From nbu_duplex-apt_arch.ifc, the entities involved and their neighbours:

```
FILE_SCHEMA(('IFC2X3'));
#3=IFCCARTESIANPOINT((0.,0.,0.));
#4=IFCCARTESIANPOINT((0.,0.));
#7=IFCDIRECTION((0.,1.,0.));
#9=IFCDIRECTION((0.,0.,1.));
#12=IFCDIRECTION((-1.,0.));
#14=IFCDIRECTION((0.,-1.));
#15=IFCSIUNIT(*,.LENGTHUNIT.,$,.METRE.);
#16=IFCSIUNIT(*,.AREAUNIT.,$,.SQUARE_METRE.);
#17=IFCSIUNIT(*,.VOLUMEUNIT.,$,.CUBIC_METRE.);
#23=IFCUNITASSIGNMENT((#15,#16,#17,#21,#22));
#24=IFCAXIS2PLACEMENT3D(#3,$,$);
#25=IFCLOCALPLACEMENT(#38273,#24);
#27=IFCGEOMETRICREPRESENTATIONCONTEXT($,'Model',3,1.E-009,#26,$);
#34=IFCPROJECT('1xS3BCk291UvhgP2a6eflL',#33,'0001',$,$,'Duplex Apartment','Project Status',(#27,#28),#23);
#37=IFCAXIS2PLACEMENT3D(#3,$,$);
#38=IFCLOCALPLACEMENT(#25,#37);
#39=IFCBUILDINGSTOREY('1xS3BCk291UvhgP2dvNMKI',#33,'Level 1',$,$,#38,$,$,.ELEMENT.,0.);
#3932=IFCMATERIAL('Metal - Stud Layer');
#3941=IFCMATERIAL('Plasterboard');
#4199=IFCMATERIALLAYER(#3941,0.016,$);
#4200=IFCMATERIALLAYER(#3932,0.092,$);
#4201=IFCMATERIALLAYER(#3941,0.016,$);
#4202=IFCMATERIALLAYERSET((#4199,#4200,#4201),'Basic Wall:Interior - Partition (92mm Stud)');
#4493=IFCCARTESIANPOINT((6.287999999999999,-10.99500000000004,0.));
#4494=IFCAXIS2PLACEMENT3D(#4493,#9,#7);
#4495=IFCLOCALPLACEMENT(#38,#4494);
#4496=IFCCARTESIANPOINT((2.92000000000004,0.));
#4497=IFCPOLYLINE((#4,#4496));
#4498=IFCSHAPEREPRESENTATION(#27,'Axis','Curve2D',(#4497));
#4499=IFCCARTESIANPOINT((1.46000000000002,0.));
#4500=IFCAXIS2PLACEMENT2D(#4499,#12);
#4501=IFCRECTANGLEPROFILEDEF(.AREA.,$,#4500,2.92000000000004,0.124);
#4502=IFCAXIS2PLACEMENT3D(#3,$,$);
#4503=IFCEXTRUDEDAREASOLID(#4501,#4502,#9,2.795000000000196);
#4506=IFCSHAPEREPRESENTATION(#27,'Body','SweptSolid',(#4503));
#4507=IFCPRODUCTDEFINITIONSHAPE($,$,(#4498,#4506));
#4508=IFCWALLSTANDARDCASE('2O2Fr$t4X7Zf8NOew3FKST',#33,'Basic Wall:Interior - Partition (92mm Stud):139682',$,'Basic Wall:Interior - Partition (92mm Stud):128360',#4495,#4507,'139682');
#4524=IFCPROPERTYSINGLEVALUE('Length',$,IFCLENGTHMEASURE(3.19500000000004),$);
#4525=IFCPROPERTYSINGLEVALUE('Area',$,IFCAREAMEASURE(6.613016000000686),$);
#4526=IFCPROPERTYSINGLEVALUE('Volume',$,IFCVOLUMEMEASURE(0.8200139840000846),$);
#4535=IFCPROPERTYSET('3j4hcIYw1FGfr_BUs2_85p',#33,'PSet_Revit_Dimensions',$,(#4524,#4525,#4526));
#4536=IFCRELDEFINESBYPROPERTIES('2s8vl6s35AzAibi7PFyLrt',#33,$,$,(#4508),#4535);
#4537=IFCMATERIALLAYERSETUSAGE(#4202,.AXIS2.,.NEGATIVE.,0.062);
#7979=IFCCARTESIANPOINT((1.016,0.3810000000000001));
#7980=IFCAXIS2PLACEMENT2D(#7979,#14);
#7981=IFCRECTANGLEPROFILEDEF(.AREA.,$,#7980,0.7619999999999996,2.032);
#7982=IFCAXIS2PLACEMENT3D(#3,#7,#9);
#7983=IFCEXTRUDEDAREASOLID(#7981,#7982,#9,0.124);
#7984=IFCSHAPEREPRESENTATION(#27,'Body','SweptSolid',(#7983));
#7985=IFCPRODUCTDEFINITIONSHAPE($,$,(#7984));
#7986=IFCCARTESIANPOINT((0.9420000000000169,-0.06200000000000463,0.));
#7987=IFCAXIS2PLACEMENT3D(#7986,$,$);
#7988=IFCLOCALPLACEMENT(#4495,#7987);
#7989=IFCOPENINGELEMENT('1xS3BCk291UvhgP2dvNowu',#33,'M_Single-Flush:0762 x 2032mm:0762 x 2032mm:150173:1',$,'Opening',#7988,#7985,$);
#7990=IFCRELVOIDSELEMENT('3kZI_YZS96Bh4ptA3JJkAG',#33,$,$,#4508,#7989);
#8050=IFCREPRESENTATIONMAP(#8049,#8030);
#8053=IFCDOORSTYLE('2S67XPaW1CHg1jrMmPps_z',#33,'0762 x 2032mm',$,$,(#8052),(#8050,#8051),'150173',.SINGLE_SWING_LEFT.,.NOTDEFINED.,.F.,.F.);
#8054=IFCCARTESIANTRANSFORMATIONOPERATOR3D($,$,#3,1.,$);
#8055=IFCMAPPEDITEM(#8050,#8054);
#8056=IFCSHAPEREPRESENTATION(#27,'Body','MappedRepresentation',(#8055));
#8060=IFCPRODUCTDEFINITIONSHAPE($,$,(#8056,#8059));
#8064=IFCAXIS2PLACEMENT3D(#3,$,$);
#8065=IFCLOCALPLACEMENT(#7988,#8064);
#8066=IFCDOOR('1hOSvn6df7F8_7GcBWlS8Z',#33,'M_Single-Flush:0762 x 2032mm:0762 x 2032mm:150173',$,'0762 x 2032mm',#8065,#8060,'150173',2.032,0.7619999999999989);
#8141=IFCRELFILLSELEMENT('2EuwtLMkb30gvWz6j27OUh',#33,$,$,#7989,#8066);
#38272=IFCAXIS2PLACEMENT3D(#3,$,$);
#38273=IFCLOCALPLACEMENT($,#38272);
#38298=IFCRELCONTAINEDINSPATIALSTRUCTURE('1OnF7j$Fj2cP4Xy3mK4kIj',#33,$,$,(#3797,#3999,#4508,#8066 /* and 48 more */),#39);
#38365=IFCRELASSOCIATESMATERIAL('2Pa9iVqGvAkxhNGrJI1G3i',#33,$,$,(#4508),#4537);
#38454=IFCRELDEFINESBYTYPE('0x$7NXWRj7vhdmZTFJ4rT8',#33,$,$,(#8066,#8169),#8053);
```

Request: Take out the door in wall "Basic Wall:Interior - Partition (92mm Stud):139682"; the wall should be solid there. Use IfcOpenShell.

```python
import ifcopenshell
import ifcopenshell.api.feature
import ifcopenshell.api.pset
import ifcopenshell.api.root
import ifcopenshell.geom
import ifcopenshell.util.element
import ifcopenshell.util.shape
import ifcopenshell.util.unit

model = ifcopenshell.open("nbu_duplex-apt_arch.ifc")
area_scale = ifcopenshell.util.unit.calculate_unit_scale(model, "AREAUNIT")
volume_scale = ifcopenshell.util.unit.calculate_unit_scale(model, "VOLUMEUNIT")
settings = ifcopenshell.geom.settings()


def volume(element):
    """Net volume in cubic metres, openings subtracted."""
    shape = ifcopenshell.geom.create_shape(settings, element)
    return ifcopenshell.util.shape.get_volume(shape.geometry)


door = model.by_guid("1hOSvn6df7F8_7GcBWlS8Z")
opening = door.FillsVoids[0].RelatingOpeningElement
wall = opening.VoidsElements[0].RelatingBuildingElement
before = volume(wall)

ifcopenshell.api.root.remove_product(model, product=door)
ifcopenshell.api.feature.remove_feature(model, feature=opening)

after = volume(wall)
thickness = 0.124  # wall thickness in metres

# Update the wall's stored quantities.
pset = model.by_id(ifcopenshell.util.element.get_pset(wall, "PSet_Revit_Dimensions", should_inherit=False)["id"])
ifcopenshell.api.pset.edit_pset(model, pset=pset, properties={
    "Area": model.create_entity("IfcAreaMeasure", after / thickness / area_scale),
    "Volume": model.create_entity("IfcVolumeMeasure", after / volume_scale),
})

print(f"wall volume {before:.3f} -> {after:.3f} m3")

model.write("nbu_duplex-apt_arch_updated.ifc")
```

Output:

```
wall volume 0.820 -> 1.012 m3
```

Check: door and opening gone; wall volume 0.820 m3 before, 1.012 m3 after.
